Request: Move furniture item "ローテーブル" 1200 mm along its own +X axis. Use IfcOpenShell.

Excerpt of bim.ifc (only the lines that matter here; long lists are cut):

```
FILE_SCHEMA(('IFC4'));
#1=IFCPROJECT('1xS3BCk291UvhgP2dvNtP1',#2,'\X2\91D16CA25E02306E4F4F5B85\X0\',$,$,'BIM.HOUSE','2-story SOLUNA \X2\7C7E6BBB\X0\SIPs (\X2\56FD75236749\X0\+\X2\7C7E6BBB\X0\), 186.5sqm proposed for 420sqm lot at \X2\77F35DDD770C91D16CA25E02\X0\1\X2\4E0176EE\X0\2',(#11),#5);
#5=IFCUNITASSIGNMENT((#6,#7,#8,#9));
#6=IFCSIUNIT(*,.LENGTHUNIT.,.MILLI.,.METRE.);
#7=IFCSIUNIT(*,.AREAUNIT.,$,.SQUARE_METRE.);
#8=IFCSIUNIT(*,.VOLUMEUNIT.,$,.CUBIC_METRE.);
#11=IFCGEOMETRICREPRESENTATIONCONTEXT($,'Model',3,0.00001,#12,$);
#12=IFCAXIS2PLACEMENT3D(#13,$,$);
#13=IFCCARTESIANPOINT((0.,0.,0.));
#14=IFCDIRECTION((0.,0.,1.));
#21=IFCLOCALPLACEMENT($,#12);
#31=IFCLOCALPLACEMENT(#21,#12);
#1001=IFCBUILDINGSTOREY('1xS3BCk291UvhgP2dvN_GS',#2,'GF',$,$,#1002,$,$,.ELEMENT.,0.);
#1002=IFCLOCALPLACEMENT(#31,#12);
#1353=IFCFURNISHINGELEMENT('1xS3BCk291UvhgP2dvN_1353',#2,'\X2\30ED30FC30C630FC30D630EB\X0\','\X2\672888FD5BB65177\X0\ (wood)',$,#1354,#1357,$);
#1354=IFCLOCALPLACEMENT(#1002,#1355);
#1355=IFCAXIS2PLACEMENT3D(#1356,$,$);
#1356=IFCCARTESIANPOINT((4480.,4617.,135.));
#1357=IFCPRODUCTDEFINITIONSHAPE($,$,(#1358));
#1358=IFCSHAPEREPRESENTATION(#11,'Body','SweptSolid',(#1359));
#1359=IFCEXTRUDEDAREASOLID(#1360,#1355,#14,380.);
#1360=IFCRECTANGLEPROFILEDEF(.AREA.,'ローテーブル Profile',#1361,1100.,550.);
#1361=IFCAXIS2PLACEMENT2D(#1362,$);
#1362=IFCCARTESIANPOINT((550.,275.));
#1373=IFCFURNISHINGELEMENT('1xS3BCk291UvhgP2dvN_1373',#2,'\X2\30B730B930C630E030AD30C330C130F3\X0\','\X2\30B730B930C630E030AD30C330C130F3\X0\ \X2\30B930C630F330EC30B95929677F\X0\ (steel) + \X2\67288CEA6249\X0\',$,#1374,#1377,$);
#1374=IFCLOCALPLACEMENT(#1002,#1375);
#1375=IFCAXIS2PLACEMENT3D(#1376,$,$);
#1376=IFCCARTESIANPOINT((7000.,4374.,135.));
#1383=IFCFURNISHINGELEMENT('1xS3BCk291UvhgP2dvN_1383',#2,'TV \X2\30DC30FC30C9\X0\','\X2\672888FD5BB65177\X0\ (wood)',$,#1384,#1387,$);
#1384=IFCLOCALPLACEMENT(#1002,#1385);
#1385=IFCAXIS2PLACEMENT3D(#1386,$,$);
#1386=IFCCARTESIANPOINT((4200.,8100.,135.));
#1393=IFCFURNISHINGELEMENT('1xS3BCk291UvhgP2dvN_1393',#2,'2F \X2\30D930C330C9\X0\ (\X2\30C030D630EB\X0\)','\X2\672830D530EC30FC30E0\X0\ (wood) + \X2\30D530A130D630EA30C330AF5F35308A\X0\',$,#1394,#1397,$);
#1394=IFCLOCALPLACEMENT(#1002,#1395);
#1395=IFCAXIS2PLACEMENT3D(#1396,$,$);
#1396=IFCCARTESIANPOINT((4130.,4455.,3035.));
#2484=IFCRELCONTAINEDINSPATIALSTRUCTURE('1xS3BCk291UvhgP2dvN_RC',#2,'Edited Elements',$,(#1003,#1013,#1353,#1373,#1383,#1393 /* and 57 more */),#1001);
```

```python
import ifcopenshell
import ifcopenshell.api.geometry
import ifcopenshell.util.placement

model = ifcopenshell.open("bim.ifc")

item = model.by_guid("1xS3BCk291UvhgP2dvN_1353")
matrix = ifcopenshell.util.placement.get_local_placement(item.ObjectPlacement)
matrix[:3, 3] += matrix[:3, 0] * 1200.0
ifcopenshell.api.geometry.edit_object_placement(model, product=item, matrix=matrix, is_si=False)

print(ifcopenshell.util.placement.get_local_placement(item.ObjectPlacement).round(3) + 0.0)

model.write("bim_updated.ifc")
```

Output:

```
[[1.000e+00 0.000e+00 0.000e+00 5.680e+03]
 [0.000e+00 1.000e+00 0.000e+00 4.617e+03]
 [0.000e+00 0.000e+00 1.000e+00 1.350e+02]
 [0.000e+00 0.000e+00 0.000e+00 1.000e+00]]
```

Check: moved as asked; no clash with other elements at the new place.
